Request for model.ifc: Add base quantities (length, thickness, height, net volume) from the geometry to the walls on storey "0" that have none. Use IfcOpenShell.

First a look at what the model holds.

```python
import ifcopenshell
import ifcopenshell.util.element
import ifcopenshell.util.unit

model = ifcopenshell.open("model.ifc")
print(model.schema)
for unit_type in ("LENGTHUNIT", "AREAUNIT", "VOLUMEUNIT"):
    print(unit_type, ifcopenshell.util.unit.calculate_unit_scale(model, unit_type))
storey = next(s for s in model.by_type("IfcBuildingStorey") if s.Name == "0")
walls = [e for e in ifcopenshell.util.element.get_decomposition(storey) if e.is_a("IfcWall")]
for e in sorted(walls, key=lambda e: e.id()):
    print(e.id(), e.is_a(), e.Name, list(ifcopenshell.util.element.get_psets(e, qtos_only=True)), sep=" | ")
```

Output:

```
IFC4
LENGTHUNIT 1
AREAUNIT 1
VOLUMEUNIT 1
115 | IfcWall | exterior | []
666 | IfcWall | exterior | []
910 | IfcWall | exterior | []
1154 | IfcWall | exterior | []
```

```python
import ifcopenshell
import ifcopenshell.api.pset
import ifcopenshell.geom
import ifcopenshell.util.element
import ifcopenshell.util.shape
import ifcopenshell.util.unit

model = ifcopenshell.open("model.ifc")
unit_scale = ifcopenshell.util.unit.calculate_unit_scale(model)
volume_scale = ifcopenshell.util.unit.calculate_unit_scale(model, "VOLUMEUNIT")
settings = ifcopenshell.geom.settings()

storey = next(s for s in model.by_type("IfcBuildingStorey") if s.Name == "0")
walls = [e for e in ifcopenshell.util.element.get_decomposition(storey) if e.is_a("IfcWall")]

for e in sorted(walls, key=lambda e: e.id()):
    if ifcopenshell.util.element.get_psets(e, qtos_only=True, should_inherit=False):
        continue
    # Geometry comes back in metres, in the element's own axes.
    shape = ifcopenshell.geom.create_shape(settings, e)
    values = {
        "Length": ifcopenshell.util.shape.get_x(shape.geometry) / unit_scale,
        "Width": ifcopenshell.util.shape.get_y(shape.geometry) / unit_scale,
        "Height": ifcopenshell.util.shape.get_z(shape.geometry) / unit_scale,
        "NetVolume": ifcopenshell.util.shape.get_volume(shape.geometry) / volume_scale,
    }
    qto = ifcopenshell.api.pset.add_qto(model, product=e, name="Qto_WallBaseQuantities")
    ifcopenshell.api.pset.edit_qto(model, qto=qto, properties=values)
    print(e.id(), {k: round(v, 3) for k, v in values.items()})

model.write("model_v2.ifc")
```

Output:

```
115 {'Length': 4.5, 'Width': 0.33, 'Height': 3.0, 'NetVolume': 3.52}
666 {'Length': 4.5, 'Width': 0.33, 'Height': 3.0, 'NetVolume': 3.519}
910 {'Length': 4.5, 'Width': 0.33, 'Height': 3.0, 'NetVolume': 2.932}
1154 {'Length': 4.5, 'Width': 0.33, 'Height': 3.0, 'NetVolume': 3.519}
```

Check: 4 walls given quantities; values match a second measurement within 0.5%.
